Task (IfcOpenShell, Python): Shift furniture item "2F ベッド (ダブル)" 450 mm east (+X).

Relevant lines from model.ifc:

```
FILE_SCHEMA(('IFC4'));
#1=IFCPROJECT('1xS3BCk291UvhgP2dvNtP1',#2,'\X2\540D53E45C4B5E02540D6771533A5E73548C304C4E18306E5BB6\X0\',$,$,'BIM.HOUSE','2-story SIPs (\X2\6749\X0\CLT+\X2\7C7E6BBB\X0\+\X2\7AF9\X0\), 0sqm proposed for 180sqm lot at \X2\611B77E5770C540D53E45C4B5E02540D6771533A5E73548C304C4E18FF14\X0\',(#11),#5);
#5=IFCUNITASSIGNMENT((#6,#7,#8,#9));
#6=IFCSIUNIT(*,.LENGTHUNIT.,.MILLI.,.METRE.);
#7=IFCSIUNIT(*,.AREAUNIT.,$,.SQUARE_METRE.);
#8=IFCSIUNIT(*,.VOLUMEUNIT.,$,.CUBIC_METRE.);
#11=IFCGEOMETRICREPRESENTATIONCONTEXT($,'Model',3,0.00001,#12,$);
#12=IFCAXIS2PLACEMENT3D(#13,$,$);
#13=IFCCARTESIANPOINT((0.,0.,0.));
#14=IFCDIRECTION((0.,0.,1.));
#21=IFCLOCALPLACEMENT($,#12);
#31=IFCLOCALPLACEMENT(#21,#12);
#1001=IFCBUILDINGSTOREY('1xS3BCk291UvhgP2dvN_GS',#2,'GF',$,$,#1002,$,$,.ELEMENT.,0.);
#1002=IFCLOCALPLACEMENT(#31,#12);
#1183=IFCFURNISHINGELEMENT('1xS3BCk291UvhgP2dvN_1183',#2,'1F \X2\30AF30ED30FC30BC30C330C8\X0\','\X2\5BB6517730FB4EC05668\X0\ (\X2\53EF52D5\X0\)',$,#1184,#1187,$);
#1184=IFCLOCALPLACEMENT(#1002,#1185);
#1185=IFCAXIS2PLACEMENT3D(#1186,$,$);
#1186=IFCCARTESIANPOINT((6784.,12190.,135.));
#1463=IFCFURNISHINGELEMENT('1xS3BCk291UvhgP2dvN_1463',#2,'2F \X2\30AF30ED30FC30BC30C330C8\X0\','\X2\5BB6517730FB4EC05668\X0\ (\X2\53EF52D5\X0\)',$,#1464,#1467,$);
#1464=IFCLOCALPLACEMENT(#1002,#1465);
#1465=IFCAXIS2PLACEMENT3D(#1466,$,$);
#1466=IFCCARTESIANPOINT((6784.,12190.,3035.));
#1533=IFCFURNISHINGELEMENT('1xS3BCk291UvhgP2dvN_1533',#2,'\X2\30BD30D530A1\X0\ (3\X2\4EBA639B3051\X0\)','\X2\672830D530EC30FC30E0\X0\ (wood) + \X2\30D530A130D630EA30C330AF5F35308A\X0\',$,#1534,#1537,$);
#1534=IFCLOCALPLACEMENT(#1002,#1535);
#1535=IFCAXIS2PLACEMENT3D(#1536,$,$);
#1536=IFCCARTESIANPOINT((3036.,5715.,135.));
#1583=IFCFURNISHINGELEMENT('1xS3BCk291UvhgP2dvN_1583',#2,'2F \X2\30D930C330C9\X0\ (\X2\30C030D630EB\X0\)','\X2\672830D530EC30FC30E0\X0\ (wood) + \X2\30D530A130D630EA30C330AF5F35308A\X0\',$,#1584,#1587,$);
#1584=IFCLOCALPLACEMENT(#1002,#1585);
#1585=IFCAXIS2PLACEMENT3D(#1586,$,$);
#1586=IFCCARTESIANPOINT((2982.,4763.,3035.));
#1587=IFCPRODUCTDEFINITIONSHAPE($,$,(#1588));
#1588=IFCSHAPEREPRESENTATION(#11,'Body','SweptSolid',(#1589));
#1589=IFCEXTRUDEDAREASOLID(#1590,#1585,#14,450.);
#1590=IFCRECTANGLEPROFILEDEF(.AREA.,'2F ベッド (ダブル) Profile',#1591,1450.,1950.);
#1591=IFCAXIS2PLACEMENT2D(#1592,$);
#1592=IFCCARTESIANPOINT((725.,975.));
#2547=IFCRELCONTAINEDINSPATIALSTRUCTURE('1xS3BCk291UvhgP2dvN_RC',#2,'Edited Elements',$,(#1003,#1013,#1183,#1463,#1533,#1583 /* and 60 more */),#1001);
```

```python
import ifcopenshell
import ifcopenshell.api.geometry
import ifcopenshell.util.placement
import ifcopenshell.util.unit

model = ifcopenshell.open("model.ifc")
unit_scale = ifcopenshell.util.unit.calculate_unit_scale(model)

item = model.by_id(1583)
matrix = ifcopenshell.util.placement.get_local_placement(item.ObjectPlacement)
matrix[0, 3] += 0.45 / unit_scale
ifcopenshell.api.geometry.edit_object_placement(model, product=item, matrix=matrix, is_si=False)

print(ifcopenshell.util.placement.get_local_placement(item.ObjectPlacement).round(3) + 0.0)

model.write("model_edited.ifc")
```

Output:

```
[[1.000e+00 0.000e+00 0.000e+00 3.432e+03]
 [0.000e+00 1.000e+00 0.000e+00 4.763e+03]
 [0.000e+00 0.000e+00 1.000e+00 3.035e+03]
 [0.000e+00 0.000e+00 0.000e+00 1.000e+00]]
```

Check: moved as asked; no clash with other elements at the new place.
